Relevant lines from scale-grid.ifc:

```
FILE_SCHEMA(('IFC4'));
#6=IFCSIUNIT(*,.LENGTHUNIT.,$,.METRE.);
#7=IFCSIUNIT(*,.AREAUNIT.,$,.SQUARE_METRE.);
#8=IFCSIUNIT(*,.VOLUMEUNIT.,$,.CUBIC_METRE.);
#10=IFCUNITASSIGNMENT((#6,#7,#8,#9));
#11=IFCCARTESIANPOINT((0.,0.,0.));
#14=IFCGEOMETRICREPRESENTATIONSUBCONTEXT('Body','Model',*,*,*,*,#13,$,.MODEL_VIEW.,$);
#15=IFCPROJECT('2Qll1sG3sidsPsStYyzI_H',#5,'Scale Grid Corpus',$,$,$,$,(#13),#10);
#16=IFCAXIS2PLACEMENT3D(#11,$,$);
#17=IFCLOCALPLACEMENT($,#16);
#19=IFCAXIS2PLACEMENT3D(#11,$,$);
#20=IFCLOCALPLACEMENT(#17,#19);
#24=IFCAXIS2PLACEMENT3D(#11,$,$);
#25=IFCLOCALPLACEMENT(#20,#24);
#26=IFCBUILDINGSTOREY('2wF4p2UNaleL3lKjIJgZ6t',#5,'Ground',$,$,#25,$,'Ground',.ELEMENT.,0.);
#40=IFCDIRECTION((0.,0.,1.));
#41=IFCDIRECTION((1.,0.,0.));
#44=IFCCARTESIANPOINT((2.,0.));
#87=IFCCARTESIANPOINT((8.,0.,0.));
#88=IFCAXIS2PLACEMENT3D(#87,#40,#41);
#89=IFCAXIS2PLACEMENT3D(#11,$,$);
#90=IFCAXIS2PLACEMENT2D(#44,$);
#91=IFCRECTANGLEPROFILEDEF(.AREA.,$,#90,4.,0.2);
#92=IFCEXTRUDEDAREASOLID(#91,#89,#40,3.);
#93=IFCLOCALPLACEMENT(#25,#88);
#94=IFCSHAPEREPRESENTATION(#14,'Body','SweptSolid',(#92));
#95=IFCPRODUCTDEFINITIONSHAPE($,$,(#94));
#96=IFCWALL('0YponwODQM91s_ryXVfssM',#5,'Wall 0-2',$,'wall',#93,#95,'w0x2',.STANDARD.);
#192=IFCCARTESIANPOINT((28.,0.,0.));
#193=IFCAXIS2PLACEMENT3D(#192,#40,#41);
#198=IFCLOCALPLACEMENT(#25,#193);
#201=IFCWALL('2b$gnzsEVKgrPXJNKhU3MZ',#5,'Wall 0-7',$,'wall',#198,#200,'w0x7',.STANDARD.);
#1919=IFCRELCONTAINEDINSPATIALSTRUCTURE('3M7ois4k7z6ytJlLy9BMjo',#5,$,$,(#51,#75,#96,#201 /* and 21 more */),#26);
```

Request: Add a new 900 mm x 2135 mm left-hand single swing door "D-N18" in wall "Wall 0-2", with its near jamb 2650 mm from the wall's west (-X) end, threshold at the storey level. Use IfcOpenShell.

```python
import numpy as np
import ifcopenshell
import ifcopenshell.api.feature
import ifcopenshell.api.geometry
import ifcopenshell.api.root
import ifcopenshell.api.spatial
import ifcopenshell.geom
import ifcopenshell.util.element
import ifcopenshell.util.placement
import ifcopenshell.util.representation
import ifcopenshell.util.shape
import ifcopenshell.util.unit

model = ifcopenshell.open("scale-grid.ifc")
unit_scale = ifcopenshell.util.unit.calculate_unit_scale(model)
settings = ifcopenshell.geom.settings()


def volume(element):
    """Net volume in cubic metres, openings subtracted."""
    shape = ifcopenshell.geom.create_shape(settings, element)
    return ifcopenshell.util.shape.get_volume(shape.geometry)


wall = model.by_guid("0YponwODQM91s_ryXVfssM")
storey = ifcopenshell.util.element.get_container(wall, ifc_class="IfcBuildingStorey")
context = ifcopenshell.util.representation.get_context(model, "Model", "Body", "MODEL_VIEW")
before = volume(wall)

width, height, from_end, sill = 0.9, 2.135, 2.65, 0.0  # metres

# The wall runs along its own X axis, and the end named is its -X end.
wall_shape = ifcopenshell.geom.create_shape(settings, wall)
x, y, z = ifcopenshell.util.shape.get_vertices(wall_shape.geometry).T
start = x.min() + from_end
face, thickness = float(y.min()), float(y.max() - y.min())
wall_matrix = ifcopenshell.util.placement.get_local_placement(wall.ObjectPlacement)
level = ifcopenshell.util.placement.get_local_placement(storey.ObjectPlacement)[2, 3]


def in_wall(x, y):
    """Placement at x, y metres in the wall's axes, at sill height."""
    matrix = wall_matrix.copy()
    matrix[:, 3] = wall_matrix @ np.array([x / unit_scale, y / unit_scale, 0.0, 1.0])
    matrix[2, 3] = level + sill / unit_scale
    return matrix


# Opening: a box that overshoots both wall faces by 50 mm.
opening = ifcopenshell.api.root.create_entity(model, ifc_class="IfcOpeningElement", predefined_type="OPENING")
box = ifcopenshell.api.geometry.add_wall_representation(
    model, context=context, length=width, height=height, thickness=thickness + 0.1
)
ifcopenshell.api.geometry.assign_representation(model, product=opening, representation=box)
ifcopenshell.api.geometry.edit_object_placement(model, product=opening, matrix=in_wall(start, face - 0.05), is_si=False)
ifcopenshell.api.feature.add_feature(model, feature=opening, element=wall)

door = ifcopenshell.api.root.create_entity(model, ifc_class="IfcDoor", name="D-N18", predefined_type="DOOR")
door.OverallWidth, door.OverallHeight = width / unit_scale, height / unit_scale
door.OperationType = "SINGLE_SWING_LEFT"
body = ifcopenshell.api.geometry.add_door_representation(
    model,
    context=context,
    overall_width=door.OverallWidth,
    overall_height=door.OverallHeight,
    operation_type="SINGLE_SWING_LEFT",
    lining_properties={"LiningDepth": thickness / unit_scale, "ThresholdDepth": thickness / unit_scale},
)
ifcopenshell.api.geometry.assign_representation(model, product=door, representation=body)
ifcopenshell.api.spatial.assign_container(model, products=[door], relating_structure=storey)
ifcopenshell.api.feature.add_filling(model, opening=opening, element=door)

# The lining spans the wall, so the door starts at the wall face.
ifcopenshell.api.geometry.edit_object_placement(model, product=door, matrix=in_wall(start, face), is_si=False)

after = volume(wall)

print(f"wall volume {before:.3f} -> {after:.3f} m3")

model.write("scale-grid_updated.ifc")
```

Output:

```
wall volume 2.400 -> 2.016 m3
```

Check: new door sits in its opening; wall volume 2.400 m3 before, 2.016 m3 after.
